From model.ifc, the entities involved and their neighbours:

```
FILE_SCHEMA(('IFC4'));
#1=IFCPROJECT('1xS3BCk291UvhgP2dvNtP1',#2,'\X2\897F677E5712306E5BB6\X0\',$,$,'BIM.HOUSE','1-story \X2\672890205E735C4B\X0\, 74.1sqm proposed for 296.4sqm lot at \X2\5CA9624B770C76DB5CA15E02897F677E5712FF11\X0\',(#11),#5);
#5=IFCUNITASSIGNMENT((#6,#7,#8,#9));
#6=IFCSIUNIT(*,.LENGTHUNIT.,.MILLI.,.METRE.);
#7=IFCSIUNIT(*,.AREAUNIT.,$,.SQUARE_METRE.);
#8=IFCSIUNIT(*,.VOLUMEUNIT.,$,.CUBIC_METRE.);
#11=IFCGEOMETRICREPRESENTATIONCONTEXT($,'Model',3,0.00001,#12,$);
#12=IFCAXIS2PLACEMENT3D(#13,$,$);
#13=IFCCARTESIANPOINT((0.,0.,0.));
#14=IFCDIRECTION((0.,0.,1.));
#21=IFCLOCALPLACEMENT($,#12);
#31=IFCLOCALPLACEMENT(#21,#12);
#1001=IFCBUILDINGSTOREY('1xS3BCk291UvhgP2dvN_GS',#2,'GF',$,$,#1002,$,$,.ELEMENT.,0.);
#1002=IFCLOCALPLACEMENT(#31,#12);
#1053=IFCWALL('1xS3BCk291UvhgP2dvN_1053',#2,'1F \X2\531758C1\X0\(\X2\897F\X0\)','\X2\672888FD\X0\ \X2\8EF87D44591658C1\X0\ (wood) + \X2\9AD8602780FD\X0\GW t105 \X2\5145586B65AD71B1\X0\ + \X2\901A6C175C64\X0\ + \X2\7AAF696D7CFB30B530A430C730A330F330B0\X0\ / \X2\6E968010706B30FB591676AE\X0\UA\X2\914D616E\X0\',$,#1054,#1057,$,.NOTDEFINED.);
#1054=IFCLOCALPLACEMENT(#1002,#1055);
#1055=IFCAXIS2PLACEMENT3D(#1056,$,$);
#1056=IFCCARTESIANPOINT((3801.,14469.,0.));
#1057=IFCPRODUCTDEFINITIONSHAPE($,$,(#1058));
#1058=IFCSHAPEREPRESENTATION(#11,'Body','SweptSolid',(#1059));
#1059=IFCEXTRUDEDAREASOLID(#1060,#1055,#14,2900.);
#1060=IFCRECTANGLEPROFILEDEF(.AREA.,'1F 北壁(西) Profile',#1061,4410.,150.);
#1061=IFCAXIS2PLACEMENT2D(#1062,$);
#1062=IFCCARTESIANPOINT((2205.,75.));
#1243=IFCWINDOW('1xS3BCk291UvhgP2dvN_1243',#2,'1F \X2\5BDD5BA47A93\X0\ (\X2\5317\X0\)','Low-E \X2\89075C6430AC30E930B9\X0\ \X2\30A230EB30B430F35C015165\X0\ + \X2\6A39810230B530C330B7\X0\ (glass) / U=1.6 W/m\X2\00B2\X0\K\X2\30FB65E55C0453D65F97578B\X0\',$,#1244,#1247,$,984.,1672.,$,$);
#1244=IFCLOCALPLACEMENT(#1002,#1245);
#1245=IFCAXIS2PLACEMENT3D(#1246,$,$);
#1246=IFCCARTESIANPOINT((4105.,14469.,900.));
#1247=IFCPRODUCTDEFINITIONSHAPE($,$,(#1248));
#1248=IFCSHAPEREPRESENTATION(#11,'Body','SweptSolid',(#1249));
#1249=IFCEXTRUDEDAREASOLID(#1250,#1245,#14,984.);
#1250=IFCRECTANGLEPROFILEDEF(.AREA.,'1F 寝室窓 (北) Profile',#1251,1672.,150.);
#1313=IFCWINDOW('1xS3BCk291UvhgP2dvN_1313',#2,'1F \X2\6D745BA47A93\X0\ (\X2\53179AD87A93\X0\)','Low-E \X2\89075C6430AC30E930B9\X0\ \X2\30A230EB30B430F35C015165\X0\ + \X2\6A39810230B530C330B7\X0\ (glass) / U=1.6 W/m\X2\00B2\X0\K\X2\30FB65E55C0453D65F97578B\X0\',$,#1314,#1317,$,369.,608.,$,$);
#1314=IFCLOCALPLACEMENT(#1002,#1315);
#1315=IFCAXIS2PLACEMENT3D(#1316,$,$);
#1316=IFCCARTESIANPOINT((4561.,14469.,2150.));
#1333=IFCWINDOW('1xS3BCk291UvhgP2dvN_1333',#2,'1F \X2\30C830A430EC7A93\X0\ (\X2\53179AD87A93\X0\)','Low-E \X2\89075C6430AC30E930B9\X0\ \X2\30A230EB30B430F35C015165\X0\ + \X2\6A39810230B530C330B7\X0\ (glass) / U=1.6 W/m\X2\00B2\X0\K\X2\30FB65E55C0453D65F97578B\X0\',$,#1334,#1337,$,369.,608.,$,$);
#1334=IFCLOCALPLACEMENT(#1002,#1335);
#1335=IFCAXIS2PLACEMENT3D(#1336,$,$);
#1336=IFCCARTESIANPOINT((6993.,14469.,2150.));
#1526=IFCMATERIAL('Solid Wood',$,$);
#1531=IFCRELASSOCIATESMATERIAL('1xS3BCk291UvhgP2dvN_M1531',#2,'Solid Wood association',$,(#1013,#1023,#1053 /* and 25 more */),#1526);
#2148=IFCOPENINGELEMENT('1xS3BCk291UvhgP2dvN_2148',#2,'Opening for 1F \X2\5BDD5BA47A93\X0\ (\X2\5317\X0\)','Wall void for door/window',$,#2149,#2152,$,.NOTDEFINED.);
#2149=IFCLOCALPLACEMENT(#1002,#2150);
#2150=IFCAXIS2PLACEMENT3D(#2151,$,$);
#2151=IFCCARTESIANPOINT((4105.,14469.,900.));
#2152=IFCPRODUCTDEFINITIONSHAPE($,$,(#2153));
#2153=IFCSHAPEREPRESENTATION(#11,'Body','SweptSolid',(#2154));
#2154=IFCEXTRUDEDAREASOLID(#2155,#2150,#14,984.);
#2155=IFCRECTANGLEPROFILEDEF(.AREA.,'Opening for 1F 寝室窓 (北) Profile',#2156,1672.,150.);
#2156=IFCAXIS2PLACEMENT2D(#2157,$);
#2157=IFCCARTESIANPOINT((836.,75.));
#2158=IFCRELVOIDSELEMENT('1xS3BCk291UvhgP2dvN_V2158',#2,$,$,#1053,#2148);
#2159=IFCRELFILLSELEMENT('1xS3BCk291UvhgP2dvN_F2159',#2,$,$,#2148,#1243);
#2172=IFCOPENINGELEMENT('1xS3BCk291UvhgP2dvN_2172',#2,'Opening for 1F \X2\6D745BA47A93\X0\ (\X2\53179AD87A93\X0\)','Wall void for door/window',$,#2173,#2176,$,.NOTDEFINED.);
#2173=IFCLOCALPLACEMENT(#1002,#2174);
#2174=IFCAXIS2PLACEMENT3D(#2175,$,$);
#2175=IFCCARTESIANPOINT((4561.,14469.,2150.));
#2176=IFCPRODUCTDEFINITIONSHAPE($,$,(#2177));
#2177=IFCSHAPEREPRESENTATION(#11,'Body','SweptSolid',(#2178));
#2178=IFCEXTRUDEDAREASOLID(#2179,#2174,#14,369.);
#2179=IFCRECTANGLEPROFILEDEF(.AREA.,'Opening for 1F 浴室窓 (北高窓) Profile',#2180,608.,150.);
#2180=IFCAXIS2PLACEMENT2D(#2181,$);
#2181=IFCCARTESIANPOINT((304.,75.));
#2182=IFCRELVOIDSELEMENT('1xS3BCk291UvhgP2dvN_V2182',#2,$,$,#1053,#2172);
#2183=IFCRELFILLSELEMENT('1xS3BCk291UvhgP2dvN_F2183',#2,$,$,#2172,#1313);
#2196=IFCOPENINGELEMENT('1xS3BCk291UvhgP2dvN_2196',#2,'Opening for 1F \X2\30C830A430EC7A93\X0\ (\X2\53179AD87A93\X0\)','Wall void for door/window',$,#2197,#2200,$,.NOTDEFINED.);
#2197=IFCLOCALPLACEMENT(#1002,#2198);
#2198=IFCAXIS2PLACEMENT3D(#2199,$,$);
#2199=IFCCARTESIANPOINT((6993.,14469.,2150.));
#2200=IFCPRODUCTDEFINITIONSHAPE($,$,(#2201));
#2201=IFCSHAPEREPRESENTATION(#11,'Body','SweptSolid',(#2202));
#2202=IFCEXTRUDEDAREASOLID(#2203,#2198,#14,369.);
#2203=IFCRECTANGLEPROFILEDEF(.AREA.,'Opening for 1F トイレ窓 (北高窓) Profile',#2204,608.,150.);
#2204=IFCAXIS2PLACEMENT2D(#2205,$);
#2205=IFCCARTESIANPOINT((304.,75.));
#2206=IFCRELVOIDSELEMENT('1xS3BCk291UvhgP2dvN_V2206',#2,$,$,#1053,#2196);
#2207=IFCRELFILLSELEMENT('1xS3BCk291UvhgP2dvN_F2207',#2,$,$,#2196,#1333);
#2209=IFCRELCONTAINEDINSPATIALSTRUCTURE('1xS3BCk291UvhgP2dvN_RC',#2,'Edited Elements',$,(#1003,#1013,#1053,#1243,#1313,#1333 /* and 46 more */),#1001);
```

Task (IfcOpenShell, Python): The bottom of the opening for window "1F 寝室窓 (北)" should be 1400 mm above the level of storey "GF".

```python
import numpy as np
import ifcopenshell
import ifcopenshell.api.geometry
import ifcopenshell.geom
import ifcopenshell.util.element
import ifcopenshell.util.placement
import ifcopenshell.util.shape
import ifcopenshell.util.unit

model = ifcopenshell.open("model.ifc")
unit_scale = ifcopenshell.util.unit.calculate_unit_scale(model)

window = model.by_guid("1xS3BCk291UvhgP2dvN_1243")
opening = window.FillsVoids[0].RelatingOpeningElement
storey = ifcopenshell.util.element.get_container(window, ifc_class="IfcBuildingStorey")
level = ifcopenshell.util.placement.get_local_placement(storey.ObjectPlacement)[2, 3]

# The opening's origin need not be at the sill, so measure its lowest point.
shape = ifcopenshell.geom.create_shape(ifcopenshell.geom.settings(), opening)
bottom = ifcopenshell.util.shape.get_shape_bottom_elevation(shape, shape.geometry) / unit_scale
dz = level + 1.4 / unit_scale - bottom

shift = np.array([0.0, 0.0, dz])
# The window is not placed relative to its opening, so move both.
for product in (opening, window):
    matrix = ifcopenshell.util.placement.get_local_placement(product.ObjectPlacement)
    matrix[:3, 3] += shift
    ifcopenshell.api.geometry.edit_object_placement(model, product=product, matrix=matrix, is_si=False)

print(f"moved by {dz * unit_scale:+.3f} m")

model.write("model-out.ifc")
```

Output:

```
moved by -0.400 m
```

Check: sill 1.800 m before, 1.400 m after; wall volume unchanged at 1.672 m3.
